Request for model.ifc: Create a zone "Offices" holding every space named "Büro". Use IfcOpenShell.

First a look at what the model holds.

```python
import ifcopenshell

model = ifcopenshell.open("model.ifc")
print(model.schema)
seen = {}
for space in model.by_type("IfcSpace"):
    seen[space.LongName] = seen.get(space.LongName, 0) + 1
for name, count in sorted(seen.items(), key=str):
    print(count, "x", name)
print("zones:", [z.Name for z in model.by_type("IfcZone")][:20])
```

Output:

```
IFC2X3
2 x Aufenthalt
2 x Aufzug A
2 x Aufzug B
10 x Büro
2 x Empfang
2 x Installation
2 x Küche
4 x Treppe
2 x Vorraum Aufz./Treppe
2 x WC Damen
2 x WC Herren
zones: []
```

```python
import ifcopenshell
import ifcopenshell.api.group
import ifcopenshell.api.root

model = ifcopenshell.open("model.ifc")

names = {"Büro"}
spaces = [s for s in model.by_type("IfcSpace") if s.LongName in names]

zone = ifcopenshell.api.root.create_entity(model, ifc_class="IfcZone", name="Offices")
ifcopenshell.api.group.assign_group(model, products=spaces, group=zone)
print(len(spaces), "spaces in", zone.Name)

model.write("model_updated.ifc")
```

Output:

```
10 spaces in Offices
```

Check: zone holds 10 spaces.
